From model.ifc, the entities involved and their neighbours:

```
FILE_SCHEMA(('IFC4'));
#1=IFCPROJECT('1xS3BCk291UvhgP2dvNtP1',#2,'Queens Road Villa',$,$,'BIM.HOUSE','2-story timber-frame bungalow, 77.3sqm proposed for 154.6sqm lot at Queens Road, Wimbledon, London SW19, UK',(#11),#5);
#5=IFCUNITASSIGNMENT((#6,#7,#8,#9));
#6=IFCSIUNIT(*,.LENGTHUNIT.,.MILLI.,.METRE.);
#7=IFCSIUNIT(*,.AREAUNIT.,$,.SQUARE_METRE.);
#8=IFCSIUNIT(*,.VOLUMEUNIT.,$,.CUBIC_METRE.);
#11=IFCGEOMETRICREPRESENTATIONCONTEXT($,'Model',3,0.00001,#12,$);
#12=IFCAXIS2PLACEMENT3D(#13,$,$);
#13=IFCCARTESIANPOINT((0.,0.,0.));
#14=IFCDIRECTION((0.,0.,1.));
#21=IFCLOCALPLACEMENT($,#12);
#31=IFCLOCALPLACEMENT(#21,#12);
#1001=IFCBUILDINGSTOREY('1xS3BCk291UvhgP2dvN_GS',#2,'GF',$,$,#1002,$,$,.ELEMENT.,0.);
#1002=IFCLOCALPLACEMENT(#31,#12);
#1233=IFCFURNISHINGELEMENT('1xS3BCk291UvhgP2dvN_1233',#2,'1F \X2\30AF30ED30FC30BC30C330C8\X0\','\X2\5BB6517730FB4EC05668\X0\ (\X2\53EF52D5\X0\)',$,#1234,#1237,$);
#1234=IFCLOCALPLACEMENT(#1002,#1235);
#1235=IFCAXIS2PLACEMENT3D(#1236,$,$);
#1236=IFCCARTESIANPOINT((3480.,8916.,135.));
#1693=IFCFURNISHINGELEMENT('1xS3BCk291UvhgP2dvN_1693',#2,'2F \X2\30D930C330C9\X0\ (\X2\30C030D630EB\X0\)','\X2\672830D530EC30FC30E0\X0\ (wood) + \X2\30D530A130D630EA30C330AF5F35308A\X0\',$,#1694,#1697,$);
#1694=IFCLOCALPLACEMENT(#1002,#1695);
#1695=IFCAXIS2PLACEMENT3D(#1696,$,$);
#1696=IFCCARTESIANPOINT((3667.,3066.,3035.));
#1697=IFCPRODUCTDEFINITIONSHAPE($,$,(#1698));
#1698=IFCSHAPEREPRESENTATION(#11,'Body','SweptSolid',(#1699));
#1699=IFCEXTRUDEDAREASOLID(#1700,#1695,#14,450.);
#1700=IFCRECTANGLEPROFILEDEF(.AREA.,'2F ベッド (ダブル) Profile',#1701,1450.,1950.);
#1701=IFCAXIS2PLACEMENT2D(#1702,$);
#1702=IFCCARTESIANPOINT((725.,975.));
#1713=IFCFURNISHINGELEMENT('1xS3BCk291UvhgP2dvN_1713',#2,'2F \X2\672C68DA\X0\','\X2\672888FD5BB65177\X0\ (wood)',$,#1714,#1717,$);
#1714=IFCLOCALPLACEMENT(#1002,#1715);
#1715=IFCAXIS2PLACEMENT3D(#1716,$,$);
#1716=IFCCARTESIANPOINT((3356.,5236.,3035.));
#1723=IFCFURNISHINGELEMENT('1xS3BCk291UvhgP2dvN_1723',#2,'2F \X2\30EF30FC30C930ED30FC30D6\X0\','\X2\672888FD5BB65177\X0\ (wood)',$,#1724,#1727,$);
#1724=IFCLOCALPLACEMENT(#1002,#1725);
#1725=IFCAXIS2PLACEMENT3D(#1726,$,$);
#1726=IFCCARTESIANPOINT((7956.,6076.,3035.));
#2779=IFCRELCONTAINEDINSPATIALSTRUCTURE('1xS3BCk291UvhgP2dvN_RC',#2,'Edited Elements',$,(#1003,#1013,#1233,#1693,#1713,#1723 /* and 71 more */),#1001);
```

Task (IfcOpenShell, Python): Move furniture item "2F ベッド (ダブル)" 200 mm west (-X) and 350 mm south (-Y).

```python
import ifcopenshell
import ifcopenshell.api.geometry
import ifcopenshell.util.placement

model = ifcopenshell.open("model.ifc")

item = model.by_id(1693)
matrix = ifcopenshell.util.placement.get_local_placement(item.ObjectPlacement)
matrix[0, 3] -= 200.0
matrix[1, 3] -= 350.0
ifcopenshell.api.geometry.edit_object_placement(model, product=item, matrix=matrix, is_si=False)

print(ifcopenshell.util.placement.get_local_placement(item.ObjectPlacement).round(3) + 0.0)

model.write("model-out.ifc")
```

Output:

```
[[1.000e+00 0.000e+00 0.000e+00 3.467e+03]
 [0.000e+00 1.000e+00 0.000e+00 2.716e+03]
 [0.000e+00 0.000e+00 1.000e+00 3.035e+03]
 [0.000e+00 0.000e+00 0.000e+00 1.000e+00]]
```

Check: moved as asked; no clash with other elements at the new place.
